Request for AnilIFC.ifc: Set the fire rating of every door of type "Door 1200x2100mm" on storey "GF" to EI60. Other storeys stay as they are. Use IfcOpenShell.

First a look at what the model holds.

```python
import ifcopenshell
import ifcopenshell.util.element

model = ifcopenshell.open("AnilIFC.ifc")
print(model.schema)
storey = next(s for s in model.by_type("IfcBuildingStorey") if s.Name == "GF")
doors = [e for e in ifcopenshell.util.element.get_decomposition(storey) if e.is_a("IfcDoor")]
seen = {}
for e in doors:
    element_type = ifcopenshell.util.element.get_type(e)
    key = (element_type.Name if element_type != e and element_type else None, ifcopenshell.util.element.get_pset(e, "Pset_DoorCommon", "FireRating"))
    seen[key] = seen.get(key, 0) + 1
for (name, value), count in sorted(seen.items(), key=str):
    print(count, "x", name, "|", value)
```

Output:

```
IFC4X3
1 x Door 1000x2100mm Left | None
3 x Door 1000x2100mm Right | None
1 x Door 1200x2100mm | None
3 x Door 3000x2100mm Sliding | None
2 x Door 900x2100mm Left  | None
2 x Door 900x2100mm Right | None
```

```python
import ifcopenshell
import ifcopenshell.api.pset
import ifcopenshell.util.element

model = ifcopenshell.open("AnilIFC.ifc")

storey = next(s for s in model.by_type("IfcBuildingStorey") if s.Name == "GF")
doors = [e for e in ifcopenshell.util.element.get_decomposition(storey) if e.is_a("IfcDoor")]

count = 0
for e in doors:
    element_type = ifcopenshell.util.element.get_type(e)
    if element_type in (None, e) or element_type.Name != "Door 1200x2100mm":
        continue
    # add_pset returns the element's existing set when there is one.
    pset = ifcopenshell.api.pset.add_pset(model, product=e, name="Pset_DoorCommon")
    ifcopenshell.api.pset.edit_pset(model, pset=pset, properties={"FireRating": "EI60"})
    count += 1

print(count, "doors updated")

model.write("AnilIFC_updated.ifc")
```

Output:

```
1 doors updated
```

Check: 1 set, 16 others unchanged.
